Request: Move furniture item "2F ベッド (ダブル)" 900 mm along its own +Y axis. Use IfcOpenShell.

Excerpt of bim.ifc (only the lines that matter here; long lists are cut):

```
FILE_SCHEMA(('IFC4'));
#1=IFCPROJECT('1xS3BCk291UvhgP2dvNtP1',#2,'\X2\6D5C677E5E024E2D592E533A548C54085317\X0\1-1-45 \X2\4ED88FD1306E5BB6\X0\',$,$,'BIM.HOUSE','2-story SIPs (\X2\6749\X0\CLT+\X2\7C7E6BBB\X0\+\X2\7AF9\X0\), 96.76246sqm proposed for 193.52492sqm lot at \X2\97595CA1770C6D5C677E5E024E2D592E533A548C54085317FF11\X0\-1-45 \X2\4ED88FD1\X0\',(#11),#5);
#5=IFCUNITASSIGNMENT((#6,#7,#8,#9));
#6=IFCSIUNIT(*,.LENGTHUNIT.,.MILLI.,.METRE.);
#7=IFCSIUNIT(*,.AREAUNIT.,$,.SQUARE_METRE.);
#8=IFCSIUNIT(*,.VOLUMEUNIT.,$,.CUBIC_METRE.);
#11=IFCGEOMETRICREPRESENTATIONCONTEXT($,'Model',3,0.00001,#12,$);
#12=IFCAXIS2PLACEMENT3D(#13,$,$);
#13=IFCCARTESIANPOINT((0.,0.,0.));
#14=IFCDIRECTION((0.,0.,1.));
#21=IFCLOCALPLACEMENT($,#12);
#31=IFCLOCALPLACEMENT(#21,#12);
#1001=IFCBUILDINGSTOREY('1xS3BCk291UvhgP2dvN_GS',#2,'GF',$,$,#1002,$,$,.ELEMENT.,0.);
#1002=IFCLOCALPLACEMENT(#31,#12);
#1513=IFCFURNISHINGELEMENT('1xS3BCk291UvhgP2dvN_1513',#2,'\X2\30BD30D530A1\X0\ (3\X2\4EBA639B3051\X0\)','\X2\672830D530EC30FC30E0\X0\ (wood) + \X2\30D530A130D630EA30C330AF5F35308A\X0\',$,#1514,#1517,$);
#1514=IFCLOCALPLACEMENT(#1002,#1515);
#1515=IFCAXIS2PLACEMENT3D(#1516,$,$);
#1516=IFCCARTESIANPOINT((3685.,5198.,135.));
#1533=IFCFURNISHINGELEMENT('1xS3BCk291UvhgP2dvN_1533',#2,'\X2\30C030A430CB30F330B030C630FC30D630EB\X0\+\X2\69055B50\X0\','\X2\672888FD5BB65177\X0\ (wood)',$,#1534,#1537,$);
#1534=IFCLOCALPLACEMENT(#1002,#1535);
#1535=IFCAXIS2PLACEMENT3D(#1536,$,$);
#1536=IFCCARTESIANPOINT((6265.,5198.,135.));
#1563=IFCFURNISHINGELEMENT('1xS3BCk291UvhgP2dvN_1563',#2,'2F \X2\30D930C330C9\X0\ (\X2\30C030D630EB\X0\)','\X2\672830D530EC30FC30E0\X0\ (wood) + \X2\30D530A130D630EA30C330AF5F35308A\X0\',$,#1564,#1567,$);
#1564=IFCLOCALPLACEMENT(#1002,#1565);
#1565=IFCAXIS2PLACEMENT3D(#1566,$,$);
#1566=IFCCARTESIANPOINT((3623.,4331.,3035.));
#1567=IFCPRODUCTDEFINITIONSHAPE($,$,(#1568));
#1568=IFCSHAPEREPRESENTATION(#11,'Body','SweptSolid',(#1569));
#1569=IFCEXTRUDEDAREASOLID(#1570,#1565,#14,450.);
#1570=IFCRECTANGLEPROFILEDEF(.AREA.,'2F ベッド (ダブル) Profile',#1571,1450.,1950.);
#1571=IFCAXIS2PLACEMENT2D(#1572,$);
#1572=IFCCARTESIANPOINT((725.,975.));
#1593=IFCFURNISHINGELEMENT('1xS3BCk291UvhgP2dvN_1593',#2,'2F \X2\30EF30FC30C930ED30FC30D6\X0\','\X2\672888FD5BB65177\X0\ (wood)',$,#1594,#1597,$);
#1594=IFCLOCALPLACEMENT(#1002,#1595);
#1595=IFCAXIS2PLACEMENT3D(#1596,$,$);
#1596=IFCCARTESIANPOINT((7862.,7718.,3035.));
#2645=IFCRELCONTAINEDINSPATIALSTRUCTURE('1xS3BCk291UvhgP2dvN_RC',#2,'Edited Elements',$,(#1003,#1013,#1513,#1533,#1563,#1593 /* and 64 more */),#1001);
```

```python
import ifcopenshell
import ifcopenshell.api.geometry
import ifcopenshell.util.placement

model = ifcopenshell.open("bim.ifc")

item = model.by_id(1563)
matrix = ifcopenshell.util.placement.get_local_placement(item.ObjectPlacement)
matrix[:3, 3] += matrix[:3, 1] * 900.0
ifcopenshell.api.geometry.edit_object_placement(model, product=item, matrix=matrix, is_si=False)

print(ifcopenshell.util.placement.get_local_placement(item.ObjectPlacement).round(3) + 0.0)

model.write("bim_rev.ifc")
```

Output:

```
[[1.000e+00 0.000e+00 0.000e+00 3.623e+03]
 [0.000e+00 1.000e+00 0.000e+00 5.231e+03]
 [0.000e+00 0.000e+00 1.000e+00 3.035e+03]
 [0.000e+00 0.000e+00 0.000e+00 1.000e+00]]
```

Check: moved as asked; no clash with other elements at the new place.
